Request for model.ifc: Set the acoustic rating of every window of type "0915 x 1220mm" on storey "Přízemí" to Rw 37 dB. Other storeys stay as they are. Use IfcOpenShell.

First a look at what the model holds.

```python
import ifcopenshell
import ifcopenshell.util.element

model = ifcopenshell.open("model.ifc")
print(model.schema)
storey = next(s for s in model.by_type("IfcBuildingStorey") if s.Name == "Přízemí")
windows = [e for e in ifcopenshell.util.element.get_decomposition(storey) if e.is_a("IfcWindow")]
seen = {}
for e in windows:
    element_type = ifcopenshell.util.element.get_type(e)
    key = (element_type.Name if element_type != e and element_type else None, ifcopenshell.util.element.get_pset(e, "Pset_WindowCommon", "AcousticRating"))
    seen[key] = seen.get(key, 0) + 1
for (name, value), count in sorted(seen.items(), key=str):
    print(count, "x", name, "|", value)
```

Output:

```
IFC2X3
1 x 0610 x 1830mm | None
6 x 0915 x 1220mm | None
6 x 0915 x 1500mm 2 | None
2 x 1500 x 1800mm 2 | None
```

```python
import ifcopenshell
import ifcopenshell.api.pset
import ifcopenshell.util.element

model = ifcopenshell.open("model.ifc")

storey = next(s for s in model.by_type("IfcBuildingStorey") if s.Name == "Přízemí")
windows = [e for e in ifcopenshell.util.element.get_decomposition(storey) if e.is_a("IfcWindow")]

count = 0
for e in windows:
    element_type = ifcopenshell.util.element.get_type(e)
    if element_type in (None, e) or element_type.Name != "0915 x 1220mm":
        continue
    # add_pset returns the element's existing set when there is one.
    pset = ifcopenshell.api.pset.add_pset(model, product=e, name="Pset_WindowCommon")
    ifcopenshell.api.pset.edit_pset(model, pset=pset, properties={"AcousticRating": "Rw 37 dB"})
    count += 1

print(count, "windows updated")

model.write("model_rev.ifc")
```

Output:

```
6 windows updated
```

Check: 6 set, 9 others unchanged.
